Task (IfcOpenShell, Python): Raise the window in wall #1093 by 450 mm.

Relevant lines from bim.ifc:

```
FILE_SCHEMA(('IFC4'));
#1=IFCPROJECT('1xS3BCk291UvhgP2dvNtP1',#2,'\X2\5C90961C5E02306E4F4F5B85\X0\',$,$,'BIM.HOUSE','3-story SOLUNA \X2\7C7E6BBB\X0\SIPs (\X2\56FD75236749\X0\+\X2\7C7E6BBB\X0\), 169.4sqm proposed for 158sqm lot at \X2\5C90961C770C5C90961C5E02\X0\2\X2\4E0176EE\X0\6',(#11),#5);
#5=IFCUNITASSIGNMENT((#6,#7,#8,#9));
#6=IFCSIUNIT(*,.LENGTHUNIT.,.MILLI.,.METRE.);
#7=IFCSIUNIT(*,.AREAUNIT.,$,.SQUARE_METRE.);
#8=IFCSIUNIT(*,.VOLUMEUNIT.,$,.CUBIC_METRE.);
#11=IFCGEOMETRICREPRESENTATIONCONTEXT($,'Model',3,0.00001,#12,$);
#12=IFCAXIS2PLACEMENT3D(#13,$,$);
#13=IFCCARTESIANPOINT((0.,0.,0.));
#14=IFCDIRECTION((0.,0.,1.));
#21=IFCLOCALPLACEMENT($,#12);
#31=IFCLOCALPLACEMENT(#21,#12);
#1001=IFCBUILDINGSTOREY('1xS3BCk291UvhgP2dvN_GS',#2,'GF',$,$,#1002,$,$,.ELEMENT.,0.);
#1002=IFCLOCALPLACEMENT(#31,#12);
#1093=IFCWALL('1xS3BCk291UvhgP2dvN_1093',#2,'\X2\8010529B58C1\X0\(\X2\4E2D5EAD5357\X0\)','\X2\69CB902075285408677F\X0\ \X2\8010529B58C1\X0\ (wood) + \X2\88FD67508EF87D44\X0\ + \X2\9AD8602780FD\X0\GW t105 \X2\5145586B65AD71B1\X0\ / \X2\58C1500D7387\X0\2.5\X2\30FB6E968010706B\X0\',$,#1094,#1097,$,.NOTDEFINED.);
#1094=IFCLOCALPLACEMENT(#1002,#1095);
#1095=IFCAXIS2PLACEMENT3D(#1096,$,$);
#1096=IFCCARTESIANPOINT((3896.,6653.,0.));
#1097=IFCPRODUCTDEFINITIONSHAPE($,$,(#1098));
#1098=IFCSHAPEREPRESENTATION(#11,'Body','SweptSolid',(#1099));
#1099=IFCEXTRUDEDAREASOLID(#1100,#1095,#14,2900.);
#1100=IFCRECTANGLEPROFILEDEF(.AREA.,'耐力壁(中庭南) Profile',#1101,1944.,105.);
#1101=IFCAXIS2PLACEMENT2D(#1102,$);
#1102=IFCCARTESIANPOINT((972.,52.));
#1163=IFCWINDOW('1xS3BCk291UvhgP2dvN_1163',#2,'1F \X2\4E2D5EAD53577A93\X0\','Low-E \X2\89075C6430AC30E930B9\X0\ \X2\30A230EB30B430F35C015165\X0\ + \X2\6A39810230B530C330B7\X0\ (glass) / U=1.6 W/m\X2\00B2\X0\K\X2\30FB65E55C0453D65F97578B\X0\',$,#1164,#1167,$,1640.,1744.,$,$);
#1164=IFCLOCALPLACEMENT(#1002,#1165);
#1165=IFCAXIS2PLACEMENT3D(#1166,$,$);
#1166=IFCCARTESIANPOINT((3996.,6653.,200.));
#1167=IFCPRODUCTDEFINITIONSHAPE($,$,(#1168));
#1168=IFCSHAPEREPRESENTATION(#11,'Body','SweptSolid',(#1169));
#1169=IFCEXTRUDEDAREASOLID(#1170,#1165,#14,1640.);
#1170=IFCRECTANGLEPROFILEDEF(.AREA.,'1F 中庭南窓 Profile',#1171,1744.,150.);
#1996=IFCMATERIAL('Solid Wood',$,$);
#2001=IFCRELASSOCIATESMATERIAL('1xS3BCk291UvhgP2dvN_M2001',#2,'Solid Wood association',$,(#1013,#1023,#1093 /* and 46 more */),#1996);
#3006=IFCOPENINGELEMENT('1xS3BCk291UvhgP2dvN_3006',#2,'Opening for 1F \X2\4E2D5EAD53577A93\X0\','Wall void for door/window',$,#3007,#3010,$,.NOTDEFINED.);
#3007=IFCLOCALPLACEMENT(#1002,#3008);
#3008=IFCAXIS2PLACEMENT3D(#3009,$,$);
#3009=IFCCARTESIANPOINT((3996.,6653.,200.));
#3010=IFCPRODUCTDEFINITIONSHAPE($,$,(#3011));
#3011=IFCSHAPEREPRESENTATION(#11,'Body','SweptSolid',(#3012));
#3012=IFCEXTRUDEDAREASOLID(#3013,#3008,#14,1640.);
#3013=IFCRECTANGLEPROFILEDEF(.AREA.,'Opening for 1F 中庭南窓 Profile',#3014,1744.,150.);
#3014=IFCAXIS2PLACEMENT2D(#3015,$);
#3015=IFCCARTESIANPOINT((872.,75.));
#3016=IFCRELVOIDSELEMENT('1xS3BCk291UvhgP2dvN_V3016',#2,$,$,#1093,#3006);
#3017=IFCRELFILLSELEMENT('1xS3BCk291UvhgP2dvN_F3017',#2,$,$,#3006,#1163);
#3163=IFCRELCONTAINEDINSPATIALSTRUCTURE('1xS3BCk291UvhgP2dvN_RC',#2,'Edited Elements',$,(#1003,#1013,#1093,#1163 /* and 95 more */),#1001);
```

```python
import numpy as np
import ifcopenshell
import ifcopenshell.api.geometry
import ifcopenshell.util.placement
import ifcopenshell.util.unit

model = ifcopenshell.open("bim.ifc")
unit_scale = ifcopenshell.util.unit.calculate_unit_scale(model)

window = model.by_guid("1xS3BCk291UvhgP2dvN_1163")
opening = window.FillsVoids[0].RelatingOpeningElement
dz = 0.45 / unit_scale

shift = np.array([0.0, 0.0, dz])
# The window is not placed relative to its opening, so move both.
for product in (opening, window):
    matrix = ifcopenshell.util.placement.get_local_placement(product.ObjectPlacement)
    matrix[:3, 3] += shift
    ifcopenshell.api.geometry.edit_object_placement(model, product=product, matrix=matrix, is_si=False)

print(f"moved by {dz * unit_scale:+.3f} m")

model.write("bim-out.ifc")
```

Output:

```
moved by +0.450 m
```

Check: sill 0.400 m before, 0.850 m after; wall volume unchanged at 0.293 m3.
